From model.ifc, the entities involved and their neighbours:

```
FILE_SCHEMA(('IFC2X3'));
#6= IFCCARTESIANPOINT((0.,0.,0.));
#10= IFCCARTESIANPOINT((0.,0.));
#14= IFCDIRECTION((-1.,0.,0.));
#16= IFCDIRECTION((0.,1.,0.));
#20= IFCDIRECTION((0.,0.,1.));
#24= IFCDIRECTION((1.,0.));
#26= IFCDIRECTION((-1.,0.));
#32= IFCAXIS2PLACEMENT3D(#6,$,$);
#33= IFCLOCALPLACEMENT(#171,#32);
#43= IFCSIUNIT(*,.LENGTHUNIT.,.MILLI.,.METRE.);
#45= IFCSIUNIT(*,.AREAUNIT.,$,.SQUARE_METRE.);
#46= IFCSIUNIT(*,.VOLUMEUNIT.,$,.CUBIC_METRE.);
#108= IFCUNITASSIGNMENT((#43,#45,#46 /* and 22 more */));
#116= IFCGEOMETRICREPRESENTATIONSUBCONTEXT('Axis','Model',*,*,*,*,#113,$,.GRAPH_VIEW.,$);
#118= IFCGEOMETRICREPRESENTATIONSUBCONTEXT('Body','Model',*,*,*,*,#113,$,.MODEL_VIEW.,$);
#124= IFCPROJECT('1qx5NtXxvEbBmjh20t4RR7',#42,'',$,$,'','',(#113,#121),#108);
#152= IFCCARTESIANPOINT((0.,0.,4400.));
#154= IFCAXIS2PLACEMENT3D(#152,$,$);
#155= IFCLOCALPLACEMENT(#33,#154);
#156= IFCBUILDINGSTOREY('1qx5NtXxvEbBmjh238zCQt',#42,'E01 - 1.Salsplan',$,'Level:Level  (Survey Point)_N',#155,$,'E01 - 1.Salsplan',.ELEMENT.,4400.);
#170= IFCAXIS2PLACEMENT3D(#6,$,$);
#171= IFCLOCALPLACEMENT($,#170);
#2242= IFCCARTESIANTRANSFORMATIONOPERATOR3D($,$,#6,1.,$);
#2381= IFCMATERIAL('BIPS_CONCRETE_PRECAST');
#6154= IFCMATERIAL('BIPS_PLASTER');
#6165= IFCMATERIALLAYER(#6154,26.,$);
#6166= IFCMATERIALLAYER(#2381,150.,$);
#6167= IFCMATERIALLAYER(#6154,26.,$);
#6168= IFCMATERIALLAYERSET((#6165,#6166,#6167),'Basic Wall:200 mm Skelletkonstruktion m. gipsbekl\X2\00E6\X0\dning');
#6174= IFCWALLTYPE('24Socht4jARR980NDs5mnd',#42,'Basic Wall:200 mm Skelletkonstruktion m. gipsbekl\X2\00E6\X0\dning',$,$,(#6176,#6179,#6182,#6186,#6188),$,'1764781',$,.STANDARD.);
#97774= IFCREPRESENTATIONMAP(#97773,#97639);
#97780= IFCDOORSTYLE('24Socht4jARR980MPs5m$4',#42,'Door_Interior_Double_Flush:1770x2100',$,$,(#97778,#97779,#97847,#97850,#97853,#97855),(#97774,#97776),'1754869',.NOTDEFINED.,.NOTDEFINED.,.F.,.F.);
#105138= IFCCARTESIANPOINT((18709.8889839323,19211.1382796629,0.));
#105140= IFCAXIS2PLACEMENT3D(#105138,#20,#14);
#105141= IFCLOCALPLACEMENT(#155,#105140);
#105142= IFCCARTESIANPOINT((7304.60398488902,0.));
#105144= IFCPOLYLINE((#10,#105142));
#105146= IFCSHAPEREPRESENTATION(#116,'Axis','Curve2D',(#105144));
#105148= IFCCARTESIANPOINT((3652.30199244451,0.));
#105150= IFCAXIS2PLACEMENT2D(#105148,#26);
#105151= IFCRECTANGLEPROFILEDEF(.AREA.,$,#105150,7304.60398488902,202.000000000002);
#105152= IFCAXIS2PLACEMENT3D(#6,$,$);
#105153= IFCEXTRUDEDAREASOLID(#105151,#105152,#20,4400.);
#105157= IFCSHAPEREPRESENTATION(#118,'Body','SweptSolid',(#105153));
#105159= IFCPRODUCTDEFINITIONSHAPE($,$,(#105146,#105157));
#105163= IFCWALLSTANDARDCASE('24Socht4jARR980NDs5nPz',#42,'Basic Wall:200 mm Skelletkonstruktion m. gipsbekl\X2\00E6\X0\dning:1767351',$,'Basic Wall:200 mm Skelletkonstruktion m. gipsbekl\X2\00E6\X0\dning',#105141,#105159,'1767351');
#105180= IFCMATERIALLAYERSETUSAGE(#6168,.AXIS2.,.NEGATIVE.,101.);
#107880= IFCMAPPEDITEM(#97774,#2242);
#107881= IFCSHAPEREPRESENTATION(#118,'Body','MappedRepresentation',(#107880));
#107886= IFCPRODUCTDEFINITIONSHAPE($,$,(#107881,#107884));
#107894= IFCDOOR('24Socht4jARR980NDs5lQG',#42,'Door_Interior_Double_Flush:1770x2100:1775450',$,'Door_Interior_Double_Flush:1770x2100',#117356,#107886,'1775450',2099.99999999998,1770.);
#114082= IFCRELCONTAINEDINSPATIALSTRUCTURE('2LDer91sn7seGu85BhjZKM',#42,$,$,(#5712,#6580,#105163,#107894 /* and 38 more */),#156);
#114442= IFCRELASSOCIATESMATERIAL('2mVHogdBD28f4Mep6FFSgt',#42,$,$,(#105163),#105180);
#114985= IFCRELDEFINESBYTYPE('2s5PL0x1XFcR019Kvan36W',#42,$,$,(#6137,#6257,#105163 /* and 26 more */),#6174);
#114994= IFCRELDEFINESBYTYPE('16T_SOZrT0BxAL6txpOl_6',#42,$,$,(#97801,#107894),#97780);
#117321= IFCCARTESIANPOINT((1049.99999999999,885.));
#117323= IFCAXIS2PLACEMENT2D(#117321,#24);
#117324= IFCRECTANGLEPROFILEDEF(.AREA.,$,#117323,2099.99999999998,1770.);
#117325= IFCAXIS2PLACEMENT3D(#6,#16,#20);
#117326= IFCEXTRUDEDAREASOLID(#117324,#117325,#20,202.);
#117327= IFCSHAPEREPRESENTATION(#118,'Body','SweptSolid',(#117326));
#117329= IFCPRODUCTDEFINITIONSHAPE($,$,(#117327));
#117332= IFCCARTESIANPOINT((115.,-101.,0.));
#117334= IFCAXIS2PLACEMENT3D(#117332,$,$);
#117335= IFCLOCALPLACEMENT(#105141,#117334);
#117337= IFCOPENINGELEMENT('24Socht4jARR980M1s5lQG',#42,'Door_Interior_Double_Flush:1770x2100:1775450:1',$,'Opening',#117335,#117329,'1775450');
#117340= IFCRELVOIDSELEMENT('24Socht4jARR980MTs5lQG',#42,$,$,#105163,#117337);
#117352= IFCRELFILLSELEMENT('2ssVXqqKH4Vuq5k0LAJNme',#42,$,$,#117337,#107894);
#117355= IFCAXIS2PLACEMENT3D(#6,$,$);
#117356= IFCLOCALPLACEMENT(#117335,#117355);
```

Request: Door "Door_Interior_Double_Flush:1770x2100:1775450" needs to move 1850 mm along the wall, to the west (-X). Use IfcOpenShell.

```python
import ifcopenshell
import ifcopenshell.api.geometry
import ifcopenshell.util.placement

model = ifcopenshell.open("model.ifc")

door = model.by_guid("24Socht4jARR980NDs5lQG")
opening = door.FillsVoids[0].RelatingOpeningElement
wall = opening.VoidsElements[0].RelatingBuildingElement

wall_matrix = ifcopenshell.util.placement.get_local_placement(wall.ObjectPlacement)
shift = wall_matrix[:3, 0] * 1850.0
before = ifcopenshell.util.placement.get_local_placement(door.ObjectPlacement)[:3, 3].copy()

# The door is placed relative to its opening, so it follows when the opening moves.
matrix = ifcopenshell.util.placement.get_local_placement(opening.ObjectPlacement)
matrix[:3, 3] += shift
ifcopenshell.api.geometry.edit_object_placement(
    model, product=opening, matrix=matrix, is_si=False, should_transform_children=True
)

after = ifcopenshell.util.placement.get_local_placement(door.ObjectPlacement)[:3, 3]
print("door moved by", (after - before).round(3) + 0.0)

model.write("model_edited.ifc")
```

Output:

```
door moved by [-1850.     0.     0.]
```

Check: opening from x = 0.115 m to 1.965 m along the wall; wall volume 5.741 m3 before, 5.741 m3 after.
